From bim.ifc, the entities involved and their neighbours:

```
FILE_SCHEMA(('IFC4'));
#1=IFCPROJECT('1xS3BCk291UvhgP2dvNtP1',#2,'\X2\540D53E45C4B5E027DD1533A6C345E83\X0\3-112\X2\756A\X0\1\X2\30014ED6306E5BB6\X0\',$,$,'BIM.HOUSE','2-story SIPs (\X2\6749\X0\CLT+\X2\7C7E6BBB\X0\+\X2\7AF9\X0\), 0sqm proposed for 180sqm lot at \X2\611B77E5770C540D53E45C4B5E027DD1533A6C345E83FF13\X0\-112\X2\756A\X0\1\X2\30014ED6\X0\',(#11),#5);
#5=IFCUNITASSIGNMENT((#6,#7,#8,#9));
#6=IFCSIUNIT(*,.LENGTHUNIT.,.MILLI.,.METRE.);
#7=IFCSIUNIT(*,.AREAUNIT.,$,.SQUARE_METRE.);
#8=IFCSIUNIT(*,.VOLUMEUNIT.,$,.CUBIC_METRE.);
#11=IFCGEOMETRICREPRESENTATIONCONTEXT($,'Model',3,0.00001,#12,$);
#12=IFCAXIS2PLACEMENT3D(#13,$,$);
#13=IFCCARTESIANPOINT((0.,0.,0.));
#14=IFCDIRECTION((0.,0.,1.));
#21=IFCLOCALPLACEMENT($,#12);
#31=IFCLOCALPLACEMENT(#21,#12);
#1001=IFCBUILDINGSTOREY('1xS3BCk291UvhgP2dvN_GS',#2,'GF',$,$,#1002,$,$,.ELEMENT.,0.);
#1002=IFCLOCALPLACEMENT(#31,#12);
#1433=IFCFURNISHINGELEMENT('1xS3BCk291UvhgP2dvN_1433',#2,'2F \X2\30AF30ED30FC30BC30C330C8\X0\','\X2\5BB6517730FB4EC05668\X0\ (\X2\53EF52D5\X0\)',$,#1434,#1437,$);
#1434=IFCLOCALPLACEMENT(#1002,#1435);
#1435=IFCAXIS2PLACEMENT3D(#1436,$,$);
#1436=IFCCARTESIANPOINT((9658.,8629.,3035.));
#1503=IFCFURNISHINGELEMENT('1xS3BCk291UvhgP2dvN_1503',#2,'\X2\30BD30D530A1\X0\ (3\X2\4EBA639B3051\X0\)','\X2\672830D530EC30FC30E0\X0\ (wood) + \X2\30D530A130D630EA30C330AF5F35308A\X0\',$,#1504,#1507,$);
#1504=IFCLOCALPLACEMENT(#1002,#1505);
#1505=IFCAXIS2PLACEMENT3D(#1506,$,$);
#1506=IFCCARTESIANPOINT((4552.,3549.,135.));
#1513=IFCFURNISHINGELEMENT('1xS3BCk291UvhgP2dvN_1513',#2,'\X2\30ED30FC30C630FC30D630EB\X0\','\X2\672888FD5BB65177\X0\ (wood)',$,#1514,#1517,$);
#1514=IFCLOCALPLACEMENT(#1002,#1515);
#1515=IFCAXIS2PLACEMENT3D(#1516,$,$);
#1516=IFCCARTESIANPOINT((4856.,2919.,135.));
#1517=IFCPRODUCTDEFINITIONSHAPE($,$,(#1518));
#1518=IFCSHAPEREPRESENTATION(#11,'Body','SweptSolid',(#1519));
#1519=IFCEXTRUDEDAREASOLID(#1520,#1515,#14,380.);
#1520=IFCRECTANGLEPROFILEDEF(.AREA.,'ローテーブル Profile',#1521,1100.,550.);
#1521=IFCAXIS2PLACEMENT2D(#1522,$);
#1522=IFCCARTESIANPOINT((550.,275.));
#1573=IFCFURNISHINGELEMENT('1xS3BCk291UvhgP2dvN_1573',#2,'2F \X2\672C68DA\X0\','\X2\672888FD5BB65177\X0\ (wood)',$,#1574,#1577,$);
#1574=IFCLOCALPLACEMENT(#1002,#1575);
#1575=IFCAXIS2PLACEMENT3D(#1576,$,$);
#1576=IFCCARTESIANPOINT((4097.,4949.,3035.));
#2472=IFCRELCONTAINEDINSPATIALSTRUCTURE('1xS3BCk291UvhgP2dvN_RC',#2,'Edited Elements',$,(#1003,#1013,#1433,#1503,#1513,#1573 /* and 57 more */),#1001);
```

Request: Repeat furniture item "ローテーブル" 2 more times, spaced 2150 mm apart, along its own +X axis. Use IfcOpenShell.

```python
import ifcopenshell
import ifcopenshell.api.geometry
import ifcopenshell.api.root
import ifcopenshell.util.element
import ifcopenshell.util.placement
import ifcopenshell.util.unit

model = ifcopenshell.open("bim.ifc")
unit_scale = ifcopenshell.util.unit.calculate_unit_scale(model)


def reuse_history(source, copy):
    """copy_class also copies each property set's owner history, people and application; keep the originals."""
    for rel in copy.IsDefinedBy:
        if rel.is_a("IfcRelDefinesByProperties") and (history := rel.RelatingPropertyDefinition.OwnerHistory):
            rel.RelatingPropertyDefinition.OwnerHistory = source.OwnerHistory
            ifcopenshell.util.element.remove_deep2(model, history)


source = model.by_id(1513)
base = ifcopenshell.util.placement.get_local_placement(source.ObjectPlacement)
step = base[:3, 0] * 2.15 / unit_scale

for i in range(1, 3):
    copy = ifcopenshell.api.root.copy_class(model, product=source)
    copy.Representation = ifcopenshell.util.element.copy_deep(
        model, source.Representation, exclude=["IfcGeometricRepresentationContext", "IfcRepresentationMap"]
    )
    reuse_history(source, copy)
    matrix = base.copy()
    matrix[:3, 3] += i * step
    print("added at", matrix[:3, 3].round(3) + 0.0)
    ifcopenshell.api.geometry.edit_object_placement(model, product=copy, matrix=matrix, is_si=False)

model.write("bim_rev.ifc")
```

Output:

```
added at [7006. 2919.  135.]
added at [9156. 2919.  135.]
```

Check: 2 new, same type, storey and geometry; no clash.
